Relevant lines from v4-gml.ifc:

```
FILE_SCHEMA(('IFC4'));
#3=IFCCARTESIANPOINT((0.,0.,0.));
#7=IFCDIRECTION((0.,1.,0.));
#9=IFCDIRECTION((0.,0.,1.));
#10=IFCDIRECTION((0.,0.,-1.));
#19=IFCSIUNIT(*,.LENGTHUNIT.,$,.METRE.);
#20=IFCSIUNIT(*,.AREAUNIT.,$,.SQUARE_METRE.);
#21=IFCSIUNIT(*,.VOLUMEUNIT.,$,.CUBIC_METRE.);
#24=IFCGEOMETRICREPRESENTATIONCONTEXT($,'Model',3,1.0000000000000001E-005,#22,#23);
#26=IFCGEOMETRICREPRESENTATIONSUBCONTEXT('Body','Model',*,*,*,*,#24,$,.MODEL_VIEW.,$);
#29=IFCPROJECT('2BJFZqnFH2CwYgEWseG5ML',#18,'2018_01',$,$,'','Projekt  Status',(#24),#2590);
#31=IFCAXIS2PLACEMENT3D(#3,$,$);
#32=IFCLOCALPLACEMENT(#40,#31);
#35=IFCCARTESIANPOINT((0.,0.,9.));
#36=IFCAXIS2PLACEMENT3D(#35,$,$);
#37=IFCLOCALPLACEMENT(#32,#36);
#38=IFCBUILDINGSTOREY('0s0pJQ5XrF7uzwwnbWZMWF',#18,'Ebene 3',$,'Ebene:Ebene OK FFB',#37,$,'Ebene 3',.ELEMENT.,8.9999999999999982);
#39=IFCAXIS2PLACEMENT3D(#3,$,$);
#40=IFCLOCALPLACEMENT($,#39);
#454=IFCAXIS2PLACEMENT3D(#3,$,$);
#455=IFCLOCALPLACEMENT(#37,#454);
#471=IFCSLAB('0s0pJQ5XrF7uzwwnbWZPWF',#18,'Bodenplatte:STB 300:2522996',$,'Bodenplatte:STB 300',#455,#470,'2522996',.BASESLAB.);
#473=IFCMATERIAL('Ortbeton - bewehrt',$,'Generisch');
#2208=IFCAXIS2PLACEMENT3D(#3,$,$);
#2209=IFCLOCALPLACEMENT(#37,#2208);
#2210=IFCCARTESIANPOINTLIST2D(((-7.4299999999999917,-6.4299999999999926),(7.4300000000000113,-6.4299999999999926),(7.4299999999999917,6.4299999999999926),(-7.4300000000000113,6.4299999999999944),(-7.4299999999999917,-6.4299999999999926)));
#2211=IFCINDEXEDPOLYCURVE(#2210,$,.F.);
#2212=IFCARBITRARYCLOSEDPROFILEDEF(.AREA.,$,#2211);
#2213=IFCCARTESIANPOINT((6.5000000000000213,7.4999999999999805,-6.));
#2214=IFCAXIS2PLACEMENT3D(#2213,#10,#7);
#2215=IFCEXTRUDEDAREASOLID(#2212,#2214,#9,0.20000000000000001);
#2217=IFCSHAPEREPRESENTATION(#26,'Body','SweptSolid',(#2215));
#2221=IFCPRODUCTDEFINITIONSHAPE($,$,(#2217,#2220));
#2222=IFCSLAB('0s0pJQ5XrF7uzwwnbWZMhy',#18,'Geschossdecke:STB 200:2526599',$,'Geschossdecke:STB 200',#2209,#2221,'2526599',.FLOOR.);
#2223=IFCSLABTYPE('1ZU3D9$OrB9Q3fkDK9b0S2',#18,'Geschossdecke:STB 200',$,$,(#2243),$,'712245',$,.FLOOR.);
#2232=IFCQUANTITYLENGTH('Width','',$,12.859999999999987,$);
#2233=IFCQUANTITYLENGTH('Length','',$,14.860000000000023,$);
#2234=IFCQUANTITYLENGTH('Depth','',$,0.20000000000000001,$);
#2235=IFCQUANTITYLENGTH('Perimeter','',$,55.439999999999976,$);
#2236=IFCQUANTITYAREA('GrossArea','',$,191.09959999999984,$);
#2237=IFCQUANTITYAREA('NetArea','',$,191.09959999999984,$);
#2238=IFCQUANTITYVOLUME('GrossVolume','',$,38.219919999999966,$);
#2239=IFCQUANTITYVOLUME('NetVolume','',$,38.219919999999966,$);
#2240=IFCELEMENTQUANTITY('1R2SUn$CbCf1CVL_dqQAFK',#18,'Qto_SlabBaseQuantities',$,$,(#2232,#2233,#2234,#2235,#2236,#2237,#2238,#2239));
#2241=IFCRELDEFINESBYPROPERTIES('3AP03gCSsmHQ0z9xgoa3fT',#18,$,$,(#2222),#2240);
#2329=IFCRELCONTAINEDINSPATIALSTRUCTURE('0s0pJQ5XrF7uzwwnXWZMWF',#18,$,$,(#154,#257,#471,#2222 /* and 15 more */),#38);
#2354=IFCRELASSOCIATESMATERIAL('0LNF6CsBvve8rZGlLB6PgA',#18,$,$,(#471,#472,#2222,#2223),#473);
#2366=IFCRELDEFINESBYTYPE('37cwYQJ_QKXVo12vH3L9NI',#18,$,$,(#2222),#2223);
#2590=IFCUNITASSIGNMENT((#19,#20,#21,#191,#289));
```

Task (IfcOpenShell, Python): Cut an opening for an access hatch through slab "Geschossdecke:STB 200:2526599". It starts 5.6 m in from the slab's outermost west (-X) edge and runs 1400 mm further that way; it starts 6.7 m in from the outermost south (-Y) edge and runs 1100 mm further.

```python
import numpy as np
import ifcopenshell
import ifcopenshell.api.feature
import ifcopenshell.api.geometry
import ifcopenshell.api.pset
import ifcopenshell.api.root
import ifcopenshell.geom
import ifcopenshell.util.element
import ifcopenshell.util.placement
import ifcopenshell.util.representation
import ifcopenshell.util.shape
import ifcopenshell.util.unit

model = ifcopenshell.open("v4-gml.ifc")
unit_scale = ifcopenshell.util.unit.calculate_unit_scale(model)
area_scale = ifcopenshell.util.unit.calculate_unit_scale(model, "AREAUNIT")
volume_scale = ifcopenshell.util.unit.calculate_unit_scale(model, "VOLUMEUNIT")
settings = ifcopenshell.geom.settings()


def volume(element):
    """Net volume in cubic metres, openings subtracted."""
    shape = ifcopenshell.geom.create_shape(settings, element)
    return ifcopenshell.util.shape.get_volume(shape.geometry)


slab = model.by_guid("0s0pJQ5XrF7uzwwnbWZMhy")
before = volume(slab)

# Extent in the slab's own axes, in metres. The edges named are its -X and -Y sides.
slab_shape = ifcopenshell.geom.create_shape(settings, slab)
vertices = ifcopenshell.util.shape.get_vertices(slab_shape.geometry)
x_min, y_min, bottom = vertices.min(axis=0)
top = vertices[:, 2].max()

opening = ifcopenshell.api.root.create_entity(model, ifc_class="IfcOpeningElement", name="Access hatch opening", predefined_type="OPENING")
context = ifcopenshell.util.representation.get_context(model, "Model", "Body", "MODEL_VIEW")
width, depth = 1.4, 1.1
outline = [(0.0, 0.0), (width, 0.0), (width, depth), (0.0, depth), (0.0, 0.0)]
# Overshoot both faces by 50 mm so the cut is clean.
shape = ifcopenshell.api.geometry.add_slab_representation(
    model, context=context, depth=top - bottom + 0.1, polyline=outline
)
ifcopenshell.api.geometry.assign_representation(model, product=opening, representation=shape)

matrix = ifcopenshell.util.placement.get_local_placement(slab.ObjectPlacement)
matrix[:, 3] = matrix @ np.append(np.array([x_min + 5.6, y_min + 6.7, bottom - 0.05]) / unit_scale, 1.0)
ifcopenshell.api.geometry.edit_object_placement(model, product=opening, matrix=matrix, is_si=False)
ifcopenshell.api.feature.add_feature(model, feature=opening, element=slab)

after = volume(slab)

# Update the slab's stored quantities.
qto = model.by_id(ifcopenshell.util.element.get_pset(slab, "Qto_SlabBaseQuantities", should_inherit=False)["id"])
ifcopenshell.api.pset.edit_qto(model, qto=qto, properties={
    "NetArea": after / (top - bottom) / area_scale,
    "NetVolume": after / volume_scale,
})

print(f"slab volume {before:.3f} -> {after:.3f} m3")

model.write("v4-gml-out.ifc")
```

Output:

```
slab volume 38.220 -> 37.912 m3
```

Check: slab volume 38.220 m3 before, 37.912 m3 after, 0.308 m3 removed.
